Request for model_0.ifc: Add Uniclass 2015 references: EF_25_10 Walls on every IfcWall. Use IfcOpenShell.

First a look at what the model holds.

```python
import ifcopenshell

model = ifcopenshell.open("model_0.ifc")
print(model.schema)
print("classifications:", [c.Name for c in model.by_type("IfcClassification")])
for ifc_class in ("IfcDoor", "IfcRoof", "IfcStair", "IfcWall", "IfcWindow"):
    print(ifc_class, len(model.by_type(ifc_class)))
```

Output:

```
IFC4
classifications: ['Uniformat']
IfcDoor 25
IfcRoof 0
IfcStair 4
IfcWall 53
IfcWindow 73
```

```python
import ifcopenshell
import ifcopenshell.api.classification

model = ifcopenshell.open("model_0.ifc")

system = ifcopenshell.api.classification.add_classification(model, classification="Uniclass 2015")

codes = {
    "IfcWall": ("EF_25_10", "Walls"),
}
for ifc_class, (code, name) in codes.items():
    products = model.by_type(ifc_class)
    ifcopenshell.api.classification.add_reference(
        model, products=products, classification=system, identification=code, name=name
    )
    print(code, len(products))

model.write("model_0_rev.ifc")
```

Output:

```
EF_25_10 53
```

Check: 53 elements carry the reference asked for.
